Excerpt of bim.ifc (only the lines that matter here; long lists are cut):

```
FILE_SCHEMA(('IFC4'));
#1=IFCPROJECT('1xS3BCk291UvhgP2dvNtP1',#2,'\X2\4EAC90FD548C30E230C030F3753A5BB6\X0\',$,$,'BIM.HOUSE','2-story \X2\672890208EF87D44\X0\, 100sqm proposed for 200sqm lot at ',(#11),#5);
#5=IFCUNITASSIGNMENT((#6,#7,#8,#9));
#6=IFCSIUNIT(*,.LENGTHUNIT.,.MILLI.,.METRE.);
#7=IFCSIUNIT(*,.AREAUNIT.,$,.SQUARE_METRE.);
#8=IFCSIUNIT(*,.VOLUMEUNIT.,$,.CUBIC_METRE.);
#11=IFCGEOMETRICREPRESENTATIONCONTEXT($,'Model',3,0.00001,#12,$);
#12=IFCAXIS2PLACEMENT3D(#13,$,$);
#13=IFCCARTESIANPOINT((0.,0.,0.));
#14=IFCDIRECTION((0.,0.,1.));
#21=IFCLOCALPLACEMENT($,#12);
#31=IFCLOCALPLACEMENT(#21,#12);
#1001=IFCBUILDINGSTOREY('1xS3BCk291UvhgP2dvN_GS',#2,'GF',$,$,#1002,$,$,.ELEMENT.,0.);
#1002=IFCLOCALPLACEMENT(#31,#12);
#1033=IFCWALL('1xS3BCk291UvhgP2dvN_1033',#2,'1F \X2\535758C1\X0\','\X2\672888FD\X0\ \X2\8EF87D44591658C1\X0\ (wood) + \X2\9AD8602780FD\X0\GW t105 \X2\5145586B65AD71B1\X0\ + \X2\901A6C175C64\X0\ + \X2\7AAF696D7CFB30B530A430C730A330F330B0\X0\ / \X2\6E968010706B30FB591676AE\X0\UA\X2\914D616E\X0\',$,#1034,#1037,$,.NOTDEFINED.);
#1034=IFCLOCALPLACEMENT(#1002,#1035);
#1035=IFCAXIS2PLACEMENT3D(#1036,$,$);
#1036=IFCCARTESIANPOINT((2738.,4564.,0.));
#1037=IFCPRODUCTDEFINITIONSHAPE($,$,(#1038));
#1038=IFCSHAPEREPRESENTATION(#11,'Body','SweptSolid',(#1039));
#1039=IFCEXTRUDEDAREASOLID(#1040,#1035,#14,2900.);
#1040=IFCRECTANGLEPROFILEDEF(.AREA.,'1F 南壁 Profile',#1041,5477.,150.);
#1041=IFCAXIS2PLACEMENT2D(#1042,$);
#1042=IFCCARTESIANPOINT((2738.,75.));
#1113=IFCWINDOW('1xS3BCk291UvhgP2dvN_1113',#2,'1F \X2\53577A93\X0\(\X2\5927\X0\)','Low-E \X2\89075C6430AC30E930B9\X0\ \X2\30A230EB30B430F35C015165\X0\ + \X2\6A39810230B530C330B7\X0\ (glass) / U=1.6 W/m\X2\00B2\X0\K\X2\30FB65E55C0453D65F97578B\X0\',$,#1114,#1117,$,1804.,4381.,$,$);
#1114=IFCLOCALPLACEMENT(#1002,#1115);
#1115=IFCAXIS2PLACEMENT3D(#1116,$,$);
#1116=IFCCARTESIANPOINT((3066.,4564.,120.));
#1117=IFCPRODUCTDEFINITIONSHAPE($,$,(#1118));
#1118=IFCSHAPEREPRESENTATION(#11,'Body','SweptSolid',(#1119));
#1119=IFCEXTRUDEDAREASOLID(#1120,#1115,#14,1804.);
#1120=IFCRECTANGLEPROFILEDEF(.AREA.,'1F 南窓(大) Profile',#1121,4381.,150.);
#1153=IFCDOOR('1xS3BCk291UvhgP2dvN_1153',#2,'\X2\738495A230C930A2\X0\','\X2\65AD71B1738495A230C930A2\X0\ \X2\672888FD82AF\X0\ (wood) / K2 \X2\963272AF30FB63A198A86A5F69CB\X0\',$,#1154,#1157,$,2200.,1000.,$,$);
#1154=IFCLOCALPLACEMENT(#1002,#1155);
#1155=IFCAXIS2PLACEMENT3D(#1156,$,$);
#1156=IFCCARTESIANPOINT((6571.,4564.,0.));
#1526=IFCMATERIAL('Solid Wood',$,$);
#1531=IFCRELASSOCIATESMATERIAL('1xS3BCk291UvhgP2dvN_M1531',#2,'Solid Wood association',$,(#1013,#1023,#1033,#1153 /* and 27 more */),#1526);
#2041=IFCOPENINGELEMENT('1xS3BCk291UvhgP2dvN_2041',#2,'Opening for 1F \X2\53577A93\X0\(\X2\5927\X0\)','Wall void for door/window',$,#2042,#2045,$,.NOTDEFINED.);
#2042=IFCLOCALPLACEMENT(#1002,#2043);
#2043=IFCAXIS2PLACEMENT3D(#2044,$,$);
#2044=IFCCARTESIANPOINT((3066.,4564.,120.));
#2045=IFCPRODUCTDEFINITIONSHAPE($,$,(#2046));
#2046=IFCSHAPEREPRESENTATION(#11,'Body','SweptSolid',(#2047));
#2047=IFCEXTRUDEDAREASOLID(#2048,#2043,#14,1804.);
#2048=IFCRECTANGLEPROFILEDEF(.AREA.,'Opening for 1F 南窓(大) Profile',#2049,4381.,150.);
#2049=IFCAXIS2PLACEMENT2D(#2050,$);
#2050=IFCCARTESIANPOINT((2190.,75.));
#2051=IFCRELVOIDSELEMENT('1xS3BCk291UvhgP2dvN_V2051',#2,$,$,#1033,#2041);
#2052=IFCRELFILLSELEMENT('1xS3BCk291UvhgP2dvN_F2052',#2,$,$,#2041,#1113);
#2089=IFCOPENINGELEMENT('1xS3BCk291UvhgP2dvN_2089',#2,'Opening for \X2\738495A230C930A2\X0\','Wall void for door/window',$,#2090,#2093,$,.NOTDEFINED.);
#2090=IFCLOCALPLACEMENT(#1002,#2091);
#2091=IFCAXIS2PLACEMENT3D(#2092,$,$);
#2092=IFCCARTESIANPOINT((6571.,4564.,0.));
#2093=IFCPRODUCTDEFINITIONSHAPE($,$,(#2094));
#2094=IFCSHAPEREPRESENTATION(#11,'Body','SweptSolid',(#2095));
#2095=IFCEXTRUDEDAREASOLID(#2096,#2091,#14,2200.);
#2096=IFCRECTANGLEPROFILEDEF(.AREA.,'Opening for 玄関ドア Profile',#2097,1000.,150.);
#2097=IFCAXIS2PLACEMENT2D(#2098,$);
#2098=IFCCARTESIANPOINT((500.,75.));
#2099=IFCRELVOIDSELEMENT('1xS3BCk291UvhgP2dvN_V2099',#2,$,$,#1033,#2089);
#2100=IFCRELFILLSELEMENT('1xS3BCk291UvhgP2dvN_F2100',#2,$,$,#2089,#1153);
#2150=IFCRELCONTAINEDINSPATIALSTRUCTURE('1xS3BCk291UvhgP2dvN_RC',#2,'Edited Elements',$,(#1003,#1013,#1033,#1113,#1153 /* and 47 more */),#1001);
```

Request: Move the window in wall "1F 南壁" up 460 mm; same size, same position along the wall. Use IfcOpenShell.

```python
import numpy as np
import ifcopenshell
import ifcopenshell.api.geometry
import ifcopenshell.util.placement
import ifcopenshell.util.unit

model = ifcopenshell.open("bim.ifc")
unit_scale = ifcopenshell.util.unit.calculate_unit_scale(model)

window = model.by_guid("1xS3BCk291UvhgP2dvN_1113")
opening = window.FillsVoids[0].RelatingOpeningElement
dz = 0.46 / unit_scale

shift = np.array([0.0, 0.0, dz])
# The window is not placed relative to its opening, so move both.
for product in (opening, window):
    matrix = ifcopenshell.util.placement.get_local_placement(product.ObjectPlacement)
    matrix[:3, 3] += shift
    ifcopenshell.api.geometry.edit_object_placement(model, product=product, matrix=matrix, is_si=False)

print(f"moved by {dz * unit_scale:+.3f} m")

model.write("bim-out.ifc")
```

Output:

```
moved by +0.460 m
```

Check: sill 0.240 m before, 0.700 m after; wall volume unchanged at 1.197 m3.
